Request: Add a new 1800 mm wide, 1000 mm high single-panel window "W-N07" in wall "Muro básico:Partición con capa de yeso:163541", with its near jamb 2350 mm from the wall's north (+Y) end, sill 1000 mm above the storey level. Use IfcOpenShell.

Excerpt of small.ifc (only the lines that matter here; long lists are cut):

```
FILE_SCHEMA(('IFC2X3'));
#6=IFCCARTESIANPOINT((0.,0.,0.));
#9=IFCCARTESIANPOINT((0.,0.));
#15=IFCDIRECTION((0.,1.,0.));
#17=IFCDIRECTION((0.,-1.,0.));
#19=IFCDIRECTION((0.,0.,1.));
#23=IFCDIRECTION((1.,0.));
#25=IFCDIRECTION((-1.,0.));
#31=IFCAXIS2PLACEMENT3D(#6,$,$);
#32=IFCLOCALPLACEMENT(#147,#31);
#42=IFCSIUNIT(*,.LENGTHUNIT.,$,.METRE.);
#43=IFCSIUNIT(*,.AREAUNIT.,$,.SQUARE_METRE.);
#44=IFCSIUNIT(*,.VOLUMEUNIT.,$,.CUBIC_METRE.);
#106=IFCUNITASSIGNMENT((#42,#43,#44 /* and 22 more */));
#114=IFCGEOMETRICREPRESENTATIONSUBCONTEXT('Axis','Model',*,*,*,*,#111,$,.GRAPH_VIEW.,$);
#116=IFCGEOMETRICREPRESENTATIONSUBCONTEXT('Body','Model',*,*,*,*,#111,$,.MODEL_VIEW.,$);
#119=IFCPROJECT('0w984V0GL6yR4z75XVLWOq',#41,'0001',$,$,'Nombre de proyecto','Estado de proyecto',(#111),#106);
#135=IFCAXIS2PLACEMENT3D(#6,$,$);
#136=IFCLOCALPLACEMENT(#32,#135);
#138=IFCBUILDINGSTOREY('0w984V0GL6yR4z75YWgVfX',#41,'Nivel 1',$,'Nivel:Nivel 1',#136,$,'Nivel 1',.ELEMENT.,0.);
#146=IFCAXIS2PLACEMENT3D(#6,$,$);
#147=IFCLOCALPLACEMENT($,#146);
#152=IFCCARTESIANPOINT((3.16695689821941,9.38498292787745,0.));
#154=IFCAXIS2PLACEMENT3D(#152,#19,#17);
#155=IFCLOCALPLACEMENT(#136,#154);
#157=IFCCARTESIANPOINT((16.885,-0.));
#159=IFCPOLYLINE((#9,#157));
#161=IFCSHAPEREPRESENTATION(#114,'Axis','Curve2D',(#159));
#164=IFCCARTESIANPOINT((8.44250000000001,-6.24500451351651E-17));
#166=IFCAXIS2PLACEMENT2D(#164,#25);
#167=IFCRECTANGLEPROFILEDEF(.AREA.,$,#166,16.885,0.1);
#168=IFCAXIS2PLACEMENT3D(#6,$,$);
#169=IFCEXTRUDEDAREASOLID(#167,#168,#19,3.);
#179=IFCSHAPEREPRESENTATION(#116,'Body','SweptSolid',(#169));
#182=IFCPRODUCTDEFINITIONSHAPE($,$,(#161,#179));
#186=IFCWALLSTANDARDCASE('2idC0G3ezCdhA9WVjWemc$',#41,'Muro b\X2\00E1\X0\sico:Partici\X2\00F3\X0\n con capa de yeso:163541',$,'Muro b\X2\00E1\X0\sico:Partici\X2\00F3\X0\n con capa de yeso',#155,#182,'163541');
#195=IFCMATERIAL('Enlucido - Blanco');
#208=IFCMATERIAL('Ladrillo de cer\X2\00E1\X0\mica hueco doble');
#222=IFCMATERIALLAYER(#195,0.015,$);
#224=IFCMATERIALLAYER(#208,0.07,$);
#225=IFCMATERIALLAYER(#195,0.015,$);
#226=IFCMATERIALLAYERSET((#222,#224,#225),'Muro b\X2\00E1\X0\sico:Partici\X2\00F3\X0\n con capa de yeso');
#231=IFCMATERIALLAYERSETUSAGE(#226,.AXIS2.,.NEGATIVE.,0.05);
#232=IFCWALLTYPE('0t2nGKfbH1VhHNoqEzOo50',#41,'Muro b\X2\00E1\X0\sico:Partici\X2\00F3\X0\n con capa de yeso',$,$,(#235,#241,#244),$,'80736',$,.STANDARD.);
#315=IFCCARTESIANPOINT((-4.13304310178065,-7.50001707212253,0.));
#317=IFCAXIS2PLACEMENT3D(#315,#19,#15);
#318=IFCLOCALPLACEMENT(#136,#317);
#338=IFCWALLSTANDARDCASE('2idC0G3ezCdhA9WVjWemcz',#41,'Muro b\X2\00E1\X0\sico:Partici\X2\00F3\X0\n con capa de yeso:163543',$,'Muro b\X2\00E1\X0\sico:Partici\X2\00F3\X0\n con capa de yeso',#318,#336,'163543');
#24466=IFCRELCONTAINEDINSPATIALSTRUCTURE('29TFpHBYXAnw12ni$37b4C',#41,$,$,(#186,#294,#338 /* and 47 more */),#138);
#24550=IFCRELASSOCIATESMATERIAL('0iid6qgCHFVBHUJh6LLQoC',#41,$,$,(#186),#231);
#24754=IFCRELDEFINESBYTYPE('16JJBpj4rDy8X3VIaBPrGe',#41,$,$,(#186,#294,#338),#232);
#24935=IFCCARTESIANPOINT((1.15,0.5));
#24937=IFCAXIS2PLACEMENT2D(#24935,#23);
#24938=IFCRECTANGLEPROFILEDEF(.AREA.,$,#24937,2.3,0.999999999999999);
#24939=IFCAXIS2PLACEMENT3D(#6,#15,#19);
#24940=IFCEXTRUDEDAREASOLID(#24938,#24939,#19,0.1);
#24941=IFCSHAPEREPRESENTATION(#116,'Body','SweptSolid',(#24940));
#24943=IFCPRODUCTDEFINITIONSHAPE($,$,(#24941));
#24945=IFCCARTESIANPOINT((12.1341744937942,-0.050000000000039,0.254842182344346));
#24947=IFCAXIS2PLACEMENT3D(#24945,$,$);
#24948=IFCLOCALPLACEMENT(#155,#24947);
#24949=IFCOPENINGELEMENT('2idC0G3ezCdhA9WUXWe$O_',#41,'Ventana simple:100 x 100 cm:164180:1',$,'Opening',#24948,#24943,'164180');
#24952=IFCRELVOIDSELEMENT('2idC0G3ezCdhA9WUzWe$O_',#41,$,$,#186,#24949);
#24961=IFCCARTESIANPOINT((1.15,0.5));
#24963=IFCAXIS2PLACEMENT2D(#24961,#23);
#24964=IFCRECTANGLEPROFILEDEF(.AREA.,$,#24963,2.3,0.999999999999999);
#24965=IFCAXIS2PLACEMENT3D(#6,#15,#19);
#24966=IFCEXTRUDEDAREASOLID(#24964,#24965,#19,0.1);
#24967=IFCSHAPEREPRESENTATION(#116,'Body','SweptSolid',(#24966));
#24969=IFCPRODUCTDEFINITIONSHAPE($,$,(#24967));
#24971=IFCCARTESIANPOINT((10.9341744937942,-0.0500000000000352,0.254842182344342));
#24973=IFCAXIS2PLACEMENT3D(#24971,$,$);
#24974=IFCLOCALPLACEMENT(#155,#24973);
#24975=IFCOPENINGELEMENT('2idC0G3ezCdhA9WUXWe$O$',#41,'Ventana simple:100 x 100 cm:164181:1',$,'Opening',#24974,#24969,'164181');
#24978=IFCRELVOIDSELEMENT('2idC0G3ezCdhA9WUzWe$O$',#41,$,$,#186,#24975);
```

```python
import numpy as np
import ifcopenshell
import ifcopenshell.api.feature
import ifcopenshell.api.geometry
import ifcopenshell.api.root
import ifcopenshell.api.spatial
import ifcopenshell.api.type
import ifcopenshell.geom
import ifcopenshell.util.element
import ifcopenshell.util.placement
import ifcopenshell.util.representation
import ifcopenshell.util.shape
import ifcopenshell.util.unit

model = ifcopenshell.open("small.ifc")
unit_scale = ifcopenshell.util.unit.calculate_unit_scale(model)
settings = ifcopenshell.geom.settings()


def volume(element):
    """Net volume in cubic metres, openings subtracted."""
    shape = ifcopenshell.geom.create_shape(settings, element)
    return ifcopenshell.util.shape.get_volume(shape.geometry)


wall = model.by_guid("2idC0G3ezCdhA9WVjWemc$")
storey = ifcopenshell.util.element.get_container(wall, ifc_class="IfcBuildingStorey")
context = ifcopenshell.util.representation.get_context(model, "Model", "Body", "MODEL_VIEW")
before = volume(wall)

width, height, from_end, sill = 1.8, 1, 2.35, 1  # metres

# The wall runs along its own X axis, and the end named is its -X end.
wall_shape = ifcopenshell.geom.create_shape(settings, wall)
x, y, z = ifcopenshell.util.shape.get_vertices(wall_shape.geometry).T
start = x.min() + from_end
face, thickness = float(y.min()), float(y.max() - y.min())
wall_matrix = ifcopenshell.util.placement.get_local_placement(wall.ObjectPlacement)
level = ifcopenshell.util.placement.get_local_placement(storey.ObjectPlacement)[2, 3]


def in_wall(x, y):
    """Placement at x, y metres in the wall's axes, at sill height."""
    matrix = wall_matrix.copy()
    matrix[:, 3] = wall_matrix @ np.array([x / unit_scale, y / unit_scale, 0.0, 1.0])
    matrix[2, 3] = level + sill / unit_scale
    return matrix


# Opening: a box that overshoots both wall faces by 50 mm.
opening = ifcopenshell.api.root.create_entity(model, ifc_class="IfcOpeningElement")
box = ifcopenshell.api.geometry.add_wall_representation(
    model, context=context, length=width, height=height, thickness=thickness + 0.1
)
ifcopenshell.api.geometry.assign_representation(model, product=opening, representation=box)
ifcopenshell.api.geometry.edit_object_placement(model, product=opening, matrix=in_wall(start, face - 0.05), is_si=False)
ifcopenshell.api.feature.add_feature(model, feature=opening, element=wall)

window = ifcopenshell.api.root.create_entity(model, ifc_class="IfcWindow", name="W-N07")
window.OverallWidth, window.OverallHeight = width / unit_scale, height / unit_scale
body = ifcopenshell.api.geometry.add_window_representation(
    model,
    context=context,
    overall_width=window.OverallWidth,
    overall_height=window.OverallHeight,
    partition_type="SINGLE_PANEL",
)
ifcopenshell.api.geometry.assign_representation(model, product=window, representation=body)
ifcopenshell.api.spatial.assign_container(model, products=[window], relating_structure=storey)
fills = ifcopenshell.api.feature.add_filling(model, opening=opening, element=window)
fills.OwnerHistory = window.OwnerHistory  # required in IFC2X3

# IFC2X3 keeps the operation on the window style.
style = ifcopenshell.api.root.create_entity(model, ifc_class="IfcWindowStyle", name="W-N07")
style.OperationType, style.ConstructionType = "SINGLE_PANEL", "NOTDEFINED"
style.ParameterTakesPrecedence = style.Sizeable = False
ifcopenshell.api.type.assign_type(model, related_objects=[window], relating_type=style)

# Centre the window in the wall's thickness.
ifcopenshell.api.geometry.edit_object_placement(model, product=window, matrix=in_wall(start, face), is_si=False)
window_shape = ifcopenshell.geom.create_shape(settings, window)
depth = ifcopenshell.util.shape.get_vertices(window_shape.geometry)[:, 1]
offset = face + thickness / 2 - (depth.min() + depth.max()) / 2
ifcopenshell.api.geometry.edit_object_placement(model, product=window, matrix=in_wall(start, offset), is_si=False)

after = volume(wall)

print(f"wall volume {before:.3f} -> {after:.3f} m3")

model.write("small-out.ifc")
```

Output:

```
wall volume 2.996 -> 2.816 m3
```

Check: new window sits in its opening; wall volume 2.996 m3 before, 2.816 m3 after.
